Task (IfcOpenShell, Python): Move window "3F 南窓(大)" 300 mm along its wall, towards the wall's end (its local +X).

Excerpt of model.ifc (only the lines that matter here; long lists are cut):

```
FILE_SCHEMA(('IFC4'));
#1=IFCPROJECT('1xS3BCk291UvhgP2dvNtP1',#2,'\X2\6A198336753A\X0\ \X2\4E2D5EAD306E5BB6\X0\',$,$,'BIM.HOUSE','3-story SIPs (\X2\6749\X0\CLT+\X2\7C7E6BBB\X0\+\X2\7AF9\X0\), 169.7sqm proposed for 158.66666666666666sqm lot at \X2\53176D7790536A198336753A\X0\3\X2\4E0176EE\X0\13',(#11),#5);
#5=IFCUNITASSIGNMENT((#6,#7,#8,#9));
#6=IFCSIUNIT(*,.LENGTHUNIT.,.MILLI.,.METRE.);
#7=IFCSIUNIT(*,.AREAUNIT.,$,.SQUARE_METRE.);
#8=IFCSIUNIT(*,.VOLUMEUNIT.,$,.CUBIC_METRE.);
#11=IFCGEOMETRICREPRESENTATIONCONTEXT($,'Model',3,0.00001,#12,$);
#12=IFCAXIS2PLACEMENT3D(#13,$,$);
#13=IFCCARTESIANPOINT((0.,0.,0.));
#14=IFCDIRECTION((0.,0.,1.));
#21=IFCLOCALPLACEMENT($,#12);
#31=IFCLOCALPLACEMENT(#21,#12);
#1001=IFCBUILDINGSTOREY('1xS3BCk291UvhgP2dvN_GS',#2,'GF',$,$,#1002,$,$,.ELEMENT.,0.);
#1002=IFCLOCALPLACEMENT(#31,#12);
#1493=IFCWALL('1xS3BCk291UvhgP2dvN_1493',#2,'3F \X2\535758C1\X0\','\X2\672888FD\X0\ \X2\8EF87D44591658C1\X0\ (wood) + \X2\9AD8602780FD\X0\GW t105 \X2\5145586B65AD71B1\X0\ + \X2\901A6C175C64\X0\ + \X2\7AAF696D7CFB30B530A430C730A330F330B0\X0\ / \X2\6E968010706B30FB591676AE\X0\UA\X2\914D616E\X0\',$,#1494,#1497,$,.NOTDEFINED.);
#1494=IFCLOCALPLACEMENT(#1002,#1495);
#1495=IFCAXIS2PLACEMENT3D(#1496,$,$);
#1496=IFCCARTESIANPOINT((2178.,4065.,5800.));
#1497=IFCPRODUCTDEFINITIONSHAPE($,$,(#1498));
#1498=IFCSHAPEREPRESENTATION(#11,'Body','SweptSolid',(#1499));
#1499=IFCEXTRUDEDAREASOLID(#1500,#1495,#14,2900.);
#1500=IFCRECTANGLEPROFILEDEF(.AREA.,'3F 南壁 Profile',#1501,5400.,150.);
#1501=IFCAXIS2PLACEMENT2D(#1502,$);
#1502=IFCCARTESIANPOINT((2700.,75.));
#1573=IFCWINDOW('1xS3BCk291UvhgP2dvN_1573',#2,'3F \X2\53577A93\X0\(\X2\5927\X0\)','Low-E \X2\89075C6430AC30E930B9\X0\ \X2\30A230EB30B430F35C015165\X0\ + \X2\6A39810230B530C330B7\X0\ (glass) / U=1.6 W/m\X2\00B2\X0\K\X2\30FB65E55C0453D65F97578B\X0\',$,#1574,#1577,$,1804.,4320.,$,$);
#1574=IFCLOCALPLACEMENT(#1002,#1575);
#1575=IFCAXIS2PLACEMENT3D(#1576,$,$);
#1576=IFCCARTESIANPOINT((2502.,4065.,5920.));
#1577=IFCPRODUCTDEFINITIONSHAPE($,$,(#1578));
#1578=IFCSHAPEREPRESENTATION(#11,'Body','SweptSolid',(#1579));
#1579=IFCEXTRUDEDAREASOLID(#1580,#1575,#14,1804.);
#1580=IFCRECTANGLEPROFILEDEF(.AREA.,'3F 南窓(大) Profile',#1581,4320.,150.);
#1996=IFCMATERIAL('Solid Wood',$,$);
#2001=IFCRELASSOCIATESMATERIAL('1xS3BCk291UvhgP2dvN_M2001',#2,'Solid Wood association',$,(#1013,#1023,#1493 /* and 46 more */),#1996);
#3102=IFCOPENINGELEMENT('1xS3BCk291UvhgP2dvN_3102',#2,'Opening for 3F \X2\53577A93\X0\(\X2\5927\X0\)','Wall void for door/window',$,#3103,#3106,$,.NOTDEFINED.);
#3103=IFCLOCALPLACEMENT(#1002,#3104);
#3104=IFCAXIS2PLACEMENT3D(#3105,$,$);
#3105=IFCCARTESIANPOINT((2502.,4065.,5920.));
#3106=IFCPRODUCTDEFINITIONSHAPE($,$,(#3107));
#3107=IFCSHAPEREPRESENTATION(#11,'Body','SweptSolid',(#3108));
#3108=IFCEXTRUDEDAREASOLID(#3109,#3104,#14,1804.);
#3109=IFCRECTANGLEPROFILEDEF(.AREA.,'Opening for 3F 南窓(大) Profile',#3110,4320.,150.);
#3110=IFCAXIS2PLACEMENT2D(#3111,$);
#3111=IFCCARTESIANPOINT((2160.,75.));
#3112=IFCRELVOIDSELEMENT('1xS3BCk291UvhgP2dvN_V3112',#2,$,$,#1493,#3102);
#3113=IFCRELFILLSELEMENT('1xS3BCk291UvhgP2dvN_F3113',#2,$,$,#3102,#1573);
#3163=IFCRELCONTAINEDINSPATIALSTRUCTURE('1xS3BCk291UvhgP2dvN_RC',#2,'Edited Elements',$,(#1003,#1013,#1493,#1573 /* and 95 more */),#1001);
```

```python
import ifcopenshell
import ifcopenshell.api.geometry
import ifcopenshell.util.placement
import ifcopenshell.util.unit

model = ifcopenshell.open("model.ifc")
unit_scale = ifcopenshell.util.unit.calculate_unit_scale(model)

window = model.by_guid("1xS3BCk291UvhgP2dvN_1573")
opening = window.FillsVoids[0].RelatingOpeningElement
wall = opening.VoidsElements[0].RelatingBuildingElement

wall_matrix = ifcopenshell.util.placement.get_local_placement(wall.ObjectPlacement)
shift = wall_matrix[:3, 0] * 0.3 / unit_scale
before = ifcopenshell.util.placement.get_local_placement(window.ObjectPlacement)[:3, 3].copy()

# The window is not placed relative to its opening, so move both.
for product in (opening, window):
    matrix = ifcopenshell.util.placement.get_local_placement(product.ObjectPlacement)
    matrix[:3, 3] += shift
    ifcopenshell.api.geometry.edit_object_placement(model, product=product, matrix=matrix, is_si=False)

after = ifcopenshell.util.placement.get_local_placement(window.ObjectPlacement)[:3, 3]
print("window moved by", (after - before).round(3) + 0.0)

model.write("model_edited.ifc")
```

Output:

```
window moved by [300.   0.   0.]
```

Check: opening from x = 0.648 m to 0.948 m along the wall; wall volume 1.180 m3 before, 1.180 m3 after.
